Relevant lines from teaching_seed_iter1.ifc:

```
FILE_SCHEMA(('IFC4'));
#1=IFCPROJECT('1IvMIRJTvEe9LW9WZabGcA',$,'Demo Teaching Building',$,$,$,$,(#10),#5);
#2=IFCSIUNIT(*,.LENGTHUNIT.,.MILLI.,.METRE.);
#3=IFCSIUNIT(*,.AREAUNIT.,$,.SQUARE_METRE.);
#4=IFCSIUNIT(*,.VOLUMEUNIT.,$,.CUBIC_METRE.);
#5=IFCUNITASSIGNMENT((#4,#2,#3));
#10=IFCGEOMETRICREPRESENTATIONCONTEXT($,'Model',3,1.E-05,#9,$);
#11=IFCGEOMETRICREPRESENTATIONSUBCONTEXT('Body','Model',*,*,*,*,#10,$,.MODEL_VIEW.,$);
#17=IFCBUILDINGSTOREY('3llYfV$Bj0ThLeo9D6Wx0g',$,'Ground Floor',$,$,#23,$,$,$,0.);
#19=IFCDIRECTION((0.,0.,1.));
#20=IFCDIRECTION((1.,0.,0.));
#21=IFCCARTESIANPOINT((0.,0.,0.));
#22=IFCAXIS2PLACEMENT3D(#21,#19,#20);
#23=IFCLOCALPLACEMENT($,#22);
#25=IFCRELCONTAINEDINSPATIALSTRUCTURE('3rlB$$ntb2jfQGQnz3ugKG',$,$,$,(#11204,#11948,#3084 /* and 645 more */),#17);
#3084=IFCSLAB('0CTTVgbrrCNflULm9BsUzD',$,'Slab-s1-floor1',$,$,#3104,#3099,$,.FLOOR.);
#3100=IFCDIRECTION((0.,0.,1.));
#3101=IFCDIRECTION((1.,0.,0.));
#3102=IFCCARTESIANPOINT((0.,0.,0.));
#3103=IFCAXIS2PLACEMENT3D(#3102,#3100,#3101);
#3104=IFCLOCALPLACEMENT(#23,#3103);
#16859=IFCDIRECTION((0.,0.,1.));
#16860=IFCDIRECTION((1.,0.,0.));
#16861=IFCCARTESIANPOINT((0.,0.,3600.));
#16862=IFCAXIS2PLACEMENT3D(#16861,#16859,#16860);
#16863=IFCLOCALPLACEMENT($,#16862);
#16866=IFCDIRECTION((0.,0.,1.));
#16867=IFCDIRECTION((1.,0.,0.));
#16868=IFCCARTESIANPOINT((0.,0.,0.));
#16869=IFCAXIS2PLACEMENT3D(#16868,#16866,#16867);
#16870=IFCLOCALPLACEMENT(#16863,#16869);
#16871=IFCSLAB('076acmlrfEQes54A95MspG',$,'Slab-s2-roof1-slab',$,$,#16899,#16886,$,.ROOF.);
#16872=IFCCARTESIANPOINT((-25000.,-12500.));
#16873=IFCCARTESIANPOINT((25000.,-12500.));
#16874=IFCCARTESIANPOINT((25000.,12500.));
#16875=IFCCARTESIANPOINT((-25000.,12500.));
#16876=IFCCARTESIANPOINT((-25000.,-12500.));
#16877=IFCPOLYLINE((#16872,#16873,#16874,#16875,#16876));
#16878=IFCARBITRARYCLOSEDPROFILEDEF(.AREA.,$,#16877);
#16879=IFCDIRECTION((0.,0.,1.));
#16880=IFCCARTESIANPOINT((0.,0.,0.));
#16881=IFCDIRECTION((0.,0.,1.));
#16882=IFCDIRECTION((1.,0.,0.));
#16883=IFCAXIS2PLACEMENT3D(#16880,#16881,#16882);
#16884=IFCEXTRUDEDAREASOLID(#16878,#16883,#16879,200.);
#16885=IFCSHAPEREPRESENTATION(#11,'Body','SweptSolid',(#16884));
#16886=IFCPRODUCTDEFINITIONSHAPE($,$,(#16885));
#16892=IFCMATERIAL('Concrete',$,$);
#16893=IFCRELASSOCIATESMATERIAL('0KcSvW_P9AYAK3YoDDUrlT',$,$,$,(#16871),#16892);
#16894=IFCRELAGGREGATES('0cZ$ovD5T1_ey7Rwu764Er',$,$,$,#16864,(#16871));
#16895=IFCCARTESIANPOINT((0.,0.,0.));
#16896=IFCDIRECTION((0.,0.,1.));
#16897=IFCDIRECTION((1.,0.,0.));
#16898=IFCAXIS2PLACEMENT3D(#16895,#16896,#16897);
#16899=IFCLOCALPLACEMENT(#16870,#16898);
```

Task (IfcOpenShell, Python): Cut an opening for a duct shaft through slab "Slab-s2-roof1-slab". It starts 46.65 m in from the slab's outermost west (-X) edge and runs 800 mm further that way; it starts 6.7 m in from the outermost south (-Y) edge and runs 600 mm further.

```python
import numpy as np
import ifcopenshell
import ifcopenshell.api.feature
import ifcopenshell.api.geometry
import ifcopenshell.api.root
import ifcopenshell.geom
import ifcopenshell.util.placement
import ifcopenshell.util.representation
import ifcopenshell.util.shape
import ifcopenshell.util.unit

model = ifcopenshell.open("teaching_seed_iter1.ifc")
unit_scale = ifcopenshell.util.unit.calculate_unit_scale(model)
settings = ifcopenshell.geom.settings()


def volume(element):
    """Net volume in cubic metres, openings subtracted."""
    shape = ifcopenshell.geom.create_shape(settings, element)
    return ifcopenshell.util.shape.get_volume(shape.geometry)


slab = model.by_id(16871)
before = volume(slab)

# Extent in the slab's own axes, in metres. The edges named are its -X and -Y sides.
slab_shape = ifcopenshell.geom.create_shape(settings, slab)
vertices = ifcopenshell.util.shape.get_vertices(slab_shape.geometry)
x_min, y_min, bottom = vertices.min(axis=0)
top = vertices[:, 2].max()

opening = ifcopenshell.api.root.create_entity(model, ifc_class="IfcOpeningElement", name="Duct shaft opening", predefined_type="OPENING")
context = ifcopenshell.util.representation.get_context(model, "Model", "Body", "MODEL_VIEW")
width, depth = 0.8, 0.6
outline = [(0.0, 0.0), (width, 0.0), (width, depth), (0.0, depth), (0.0, 0.0)]
# Overshoot both faces by 50 mm so the cut is clean.
shape = ifcopenshell.api.geometry.add_slab_representation(
    model, context=context, depth=top - bottom + 0.1, polyline=outline
)
ifcopenshell.api.geometry.assign_representation(model, product=opening, representation=shape)

matrix = ifcopenshell.util.placement.get_local_placement(slab.ObjectPlacement)
matrix[:, 3] = matrix @ np.append(np.array([x_min + 46.65, y_min + 6.7, bottom - 0.05]) / unit_scale, 1.0)
ifcopenshell.api.geometry.edit_object_placement(model, product=opening, matrix=matrix, is_si=False)
ifcopenshell.api.feature.add_feature(model, feature=opening, element=slab)

after = volume(slab)

print(f"slab volume {before:.3f} -> {after:.3f} m3")

model.write("teaching_seed_iter1_updated.ifc")
```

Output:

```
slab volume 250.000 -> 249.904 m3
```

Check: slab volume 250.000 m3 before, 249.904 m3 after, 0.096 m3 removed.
